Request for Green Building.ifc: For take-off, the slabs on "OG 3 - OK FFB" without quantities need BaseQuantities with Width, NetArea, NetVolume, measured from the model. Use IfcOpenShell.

First a look at what the model holds.

```python
import ifcopenshell
import ifcopenshell.util.element
import ifcopenshell.util.unit

model = ifcopenshell.open("Green Building.ifc")
print(model.schema)
for unit_type in ("LENGTHUNIT", "AREAUNIT", "VOLUMEUNIT"):
    print(unit_type, ifcopenshell.util.unit.calculate_unit_scale(model, unit_type))
storey = next(s for s in model.by_type("IfcBuildingStorey") if s.Name == "OG 3 - OK FFB")
slabs = [e for e in ifcopenshell.util.element.get_decomposition(storey) if e.is_a("IfcSlab")]
for e in sorted(slabs, key=lambda e: e.id()):
    print(e.id(), e.is_a(), e.Name, list(ifcopenshell.util.element.get_psets(e, qtos_only=True)), sep=" | ")
```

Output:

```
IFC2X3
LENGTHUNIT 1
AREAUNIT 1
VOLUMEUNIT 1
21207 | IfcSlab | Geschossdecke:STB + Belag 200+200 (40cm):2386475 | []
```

```python
import ifcopenshell
import ifcopenshell.api.pset
import ifcopenshell.geom
import ifcopenshell.util.element
import ifcopenshell.util.shape
import ifcopenshell.util.unit

model = ifcopenshell.open("Green Building.ifc")
unit_scale = ifcopenshell.util.unit.calculate_unit_scale(model)
area_scale = ifcopenshell.util.unit.calculate_unit_scale(model, "AREAUNIT")
volume_scale = ifcopenshell.util.unit.calculate_unit_scale(model, "VOLUMEUNIT")
settings = ifcopenshell.geom.settings()

storey = next(s for s in model.by_type("IfcBuildingStorey") if s.Name == "OG 3 - OK FFB")
slabs = [e for e in ifcopenshell.util.element.get_decomposition(storey) if e.is_a("IfcSlab")]

for e in sorted(slabs, key=lambda e: e.id()):
    if ifcopenshell.util.element.get_psets(e, qtos_only=True, should_inherit=False):
        continue
    # Geometry comes back in metres, in the element's own axes.
    shape = ifcopenshell.geom.create_shape(settings, e)
    values = {
        "Width": ifcopenshell.util.shape.get_z(shape.geometry) / unit_scale,
        "NetArea": ifcopenshell.util.shape.get_footprint_area(shape.geometry) / area_scale,
        "NetVolume": ifcopenshell.util.shape.get_volume(shape.geometry) / volume_scale,
    }
    qto = ifcopenshell.api.pset.add_qto(model, product=e, name="BaseQuantities")
    ifcopenshell.api.pset.edit_qto(model, qto=qto, properties=values)
    print(e.id(), {k: round(v, 3) for k, v in values.items()})

model.write("Green Building-out.ifc")
```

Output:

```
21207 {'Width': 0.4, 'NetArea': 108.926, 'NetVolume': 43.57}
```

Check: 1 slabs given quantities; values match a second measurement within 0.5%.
